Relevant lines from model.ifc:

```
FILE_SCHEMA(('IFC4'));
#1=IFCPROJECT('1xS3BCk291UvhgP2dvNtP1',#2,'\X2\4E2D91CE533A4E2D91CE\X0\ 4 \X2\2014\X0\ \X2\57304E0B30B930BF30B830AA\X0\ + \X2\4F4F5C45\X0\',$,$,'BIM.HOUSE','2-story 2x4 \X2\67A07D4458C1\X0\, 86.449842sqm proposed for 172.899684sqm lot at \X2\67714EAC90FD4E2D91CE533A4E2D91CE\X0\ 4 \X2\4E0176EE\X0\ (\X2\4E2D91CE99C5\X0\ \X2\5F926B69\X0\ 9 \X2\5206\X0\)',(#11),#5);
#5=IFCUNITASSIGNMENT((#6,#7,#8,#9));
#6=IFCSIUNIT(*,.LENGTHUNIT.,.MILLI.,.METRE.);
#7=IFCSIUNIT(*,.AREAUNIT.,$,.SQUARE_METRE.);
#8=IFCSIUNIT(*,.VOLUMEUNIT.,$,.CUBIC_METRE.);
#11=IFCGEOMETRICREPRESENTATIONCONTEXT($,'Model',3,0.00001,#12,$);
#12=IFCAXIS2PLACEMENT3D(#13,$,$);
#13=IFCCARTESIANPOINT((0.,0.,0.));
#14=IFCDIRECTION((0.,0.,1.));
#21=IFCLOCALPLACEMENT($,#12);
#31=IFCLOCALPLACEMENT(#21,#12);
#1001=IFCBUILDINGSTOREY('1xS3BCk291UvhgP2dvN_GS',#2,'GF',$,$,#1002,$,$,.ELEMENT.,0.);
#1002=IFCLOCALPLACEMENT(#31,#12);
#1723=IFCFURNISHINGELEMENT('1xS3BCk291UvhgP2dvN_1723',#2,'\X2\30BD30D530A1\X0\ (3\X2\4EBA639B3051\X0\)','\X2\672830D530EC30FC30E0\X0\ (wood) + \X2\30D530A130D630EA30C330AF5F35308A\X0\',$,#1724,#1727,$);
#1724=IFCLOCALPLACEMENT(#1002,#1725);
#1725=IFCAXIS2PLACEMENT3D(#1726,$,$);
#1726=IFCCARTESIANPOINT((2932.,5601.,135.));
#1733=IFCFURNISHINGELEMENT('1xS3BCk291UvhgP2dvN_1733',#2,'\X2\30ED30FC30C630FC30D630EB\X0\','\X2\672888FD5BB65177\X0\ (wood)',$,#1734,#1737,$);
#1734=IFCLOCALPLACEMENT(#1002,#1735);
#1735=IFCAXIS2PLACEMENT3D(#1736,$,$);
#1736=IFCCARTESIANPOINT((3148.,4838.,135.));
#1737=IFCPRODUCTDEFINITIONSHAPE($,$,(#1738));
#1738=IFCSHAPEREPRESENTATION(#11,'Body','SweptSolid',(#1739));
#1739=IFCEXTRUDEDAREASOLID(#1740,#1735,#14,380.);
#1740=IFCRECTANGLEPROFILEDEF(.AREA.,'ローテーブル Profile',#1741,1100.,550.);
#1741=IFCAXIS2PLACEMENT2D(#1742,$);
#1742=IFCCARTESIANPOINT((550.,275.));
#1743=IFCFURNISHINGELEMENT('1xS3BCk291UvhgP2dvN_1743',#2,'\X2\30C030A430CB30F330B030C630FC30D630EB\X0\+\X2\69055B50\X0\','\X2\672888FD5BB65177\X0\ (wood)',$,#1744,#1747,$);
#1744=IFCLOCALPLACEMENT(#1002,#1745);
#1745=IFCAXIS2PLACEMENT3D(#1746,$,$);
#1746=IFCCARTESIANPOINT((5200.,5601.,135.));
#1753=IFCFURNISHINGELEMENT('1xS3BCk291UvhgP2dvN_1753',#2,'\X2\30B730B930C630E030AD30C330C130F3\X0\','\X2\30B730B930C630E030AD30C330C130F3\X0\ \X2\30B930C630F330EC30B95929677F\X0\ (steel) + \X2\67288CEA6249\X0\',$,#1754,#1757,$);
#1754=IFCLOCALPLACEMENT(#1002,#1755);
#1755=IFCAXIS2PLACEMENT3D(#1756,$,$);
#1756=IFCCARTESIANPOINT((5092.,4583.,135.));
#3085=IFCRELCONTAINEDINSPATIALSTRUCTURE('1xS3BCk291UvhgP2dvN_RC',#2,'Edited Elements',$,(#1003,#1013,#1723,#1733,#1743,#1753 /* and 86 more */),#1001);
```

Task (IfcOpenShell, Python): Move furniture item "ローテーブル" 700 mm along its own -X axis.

```python
import ifcopenshell
import ifcopenshell.api.geometry
import ifcopenshell.util.placement
import ifcopenshell.util.unit

model = ifcopenshell.open("model.ifc")
unit_scale = ifcopenshell.util.unit.calculate_unit_scale(model)

item = model.by_id(1733)
matrix = ifcopenshell.util.placement.get_local_placement(item.ObjectPlacement)
matrix[:3, 3] -= matrix[:3, 0] * 0.7 / unit_scale
ifcopenshell.api.geometry.edit_object_placement(model, product=item, matrix=matrix, is_si=False)

print(ifcopenshell.util.placement.get_local_placement(item.ObjectPlacement).round(3) + 0.0)

model.write("model_v2.ifc")
```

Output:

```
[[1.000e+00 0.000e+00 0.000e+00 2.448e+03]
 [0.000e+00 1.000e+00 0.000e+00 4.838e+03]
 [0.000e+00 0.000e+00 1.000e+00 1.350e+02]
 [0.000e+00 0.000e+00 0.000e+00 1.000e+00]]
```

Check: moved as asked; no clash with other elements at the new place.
